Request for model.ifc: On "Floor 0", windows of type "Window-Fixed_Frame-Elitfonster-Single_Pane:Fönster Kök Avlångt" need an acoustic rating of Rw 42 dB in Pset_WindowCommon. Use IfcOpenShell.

First a look at what the model holds.

```python
import ifcopenshell
import ifcopenshell.util.element

model = ifcopenshell.open("model.ifc")
print(model.schema)
storey = next(s for s in model.by_type("IfcBuildingStorey") if s.Name == "Floor 0")
windows = [e for e in ifcopenshell.util.element.get_decomposition(storey) if e.is_a("IfcWindow")]
seen = {}
for e in windows:
    element_type = ifcopenshell.util.element.get_type(e)
    key = (element_type.Name if element_type != e and element_type else None, ifcopenshell.util.element.get_pset(e, "Pset_WindowCommon", "AcousticRating"))
    seen[key] = seen.get(key, 0) + 1
for (name, value), count in sorted(seen.items(), key=str):
    print(count, "x", name, "|", value)
```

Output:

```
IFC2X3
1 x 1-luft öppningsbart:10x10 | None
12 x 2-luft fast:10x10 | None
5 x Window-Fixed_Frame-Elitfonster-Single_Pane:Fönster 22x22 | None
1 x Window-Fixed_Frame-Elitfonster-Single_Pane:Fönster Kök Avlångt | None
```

```python
import ifcopenshell
import ifcopenshell.api.pset
import ifcopenshell.util.element

model = ifcopenshell.open("model.ifc")

storey = next(s for s in model.by_type("IfcBuildingStorey") if s.Name == "Floor 0")
windows = [e for e in ifcopenshell.util.element.get_decomposition(storey) if e.is_a("IfcWindow")]

count = 0
for e in windows:
    element_type = ifcopenshell.util.element.get_type(e)
    if element_type in (None, e) or element_type.Name != "Window-Fixed_Frame-Elitfonster-Single_Pane:Fönster Kök Avlångt":
        continue
    # add_pset returns the element's existing set when there is one.
    pset = ifcopenshell.api.pset.add_pset(model, product=e, name="Pset_WindowCommon")
    ifcopenshell.api.pset.edit_pset(model, pset=pset, properties={"AcousticRating": "Rw 42 dB"})
    count += 1

print(count, "windows updated")

model.write("model_edited.ifc")
```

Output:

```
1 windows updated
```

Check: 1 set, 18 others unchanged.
